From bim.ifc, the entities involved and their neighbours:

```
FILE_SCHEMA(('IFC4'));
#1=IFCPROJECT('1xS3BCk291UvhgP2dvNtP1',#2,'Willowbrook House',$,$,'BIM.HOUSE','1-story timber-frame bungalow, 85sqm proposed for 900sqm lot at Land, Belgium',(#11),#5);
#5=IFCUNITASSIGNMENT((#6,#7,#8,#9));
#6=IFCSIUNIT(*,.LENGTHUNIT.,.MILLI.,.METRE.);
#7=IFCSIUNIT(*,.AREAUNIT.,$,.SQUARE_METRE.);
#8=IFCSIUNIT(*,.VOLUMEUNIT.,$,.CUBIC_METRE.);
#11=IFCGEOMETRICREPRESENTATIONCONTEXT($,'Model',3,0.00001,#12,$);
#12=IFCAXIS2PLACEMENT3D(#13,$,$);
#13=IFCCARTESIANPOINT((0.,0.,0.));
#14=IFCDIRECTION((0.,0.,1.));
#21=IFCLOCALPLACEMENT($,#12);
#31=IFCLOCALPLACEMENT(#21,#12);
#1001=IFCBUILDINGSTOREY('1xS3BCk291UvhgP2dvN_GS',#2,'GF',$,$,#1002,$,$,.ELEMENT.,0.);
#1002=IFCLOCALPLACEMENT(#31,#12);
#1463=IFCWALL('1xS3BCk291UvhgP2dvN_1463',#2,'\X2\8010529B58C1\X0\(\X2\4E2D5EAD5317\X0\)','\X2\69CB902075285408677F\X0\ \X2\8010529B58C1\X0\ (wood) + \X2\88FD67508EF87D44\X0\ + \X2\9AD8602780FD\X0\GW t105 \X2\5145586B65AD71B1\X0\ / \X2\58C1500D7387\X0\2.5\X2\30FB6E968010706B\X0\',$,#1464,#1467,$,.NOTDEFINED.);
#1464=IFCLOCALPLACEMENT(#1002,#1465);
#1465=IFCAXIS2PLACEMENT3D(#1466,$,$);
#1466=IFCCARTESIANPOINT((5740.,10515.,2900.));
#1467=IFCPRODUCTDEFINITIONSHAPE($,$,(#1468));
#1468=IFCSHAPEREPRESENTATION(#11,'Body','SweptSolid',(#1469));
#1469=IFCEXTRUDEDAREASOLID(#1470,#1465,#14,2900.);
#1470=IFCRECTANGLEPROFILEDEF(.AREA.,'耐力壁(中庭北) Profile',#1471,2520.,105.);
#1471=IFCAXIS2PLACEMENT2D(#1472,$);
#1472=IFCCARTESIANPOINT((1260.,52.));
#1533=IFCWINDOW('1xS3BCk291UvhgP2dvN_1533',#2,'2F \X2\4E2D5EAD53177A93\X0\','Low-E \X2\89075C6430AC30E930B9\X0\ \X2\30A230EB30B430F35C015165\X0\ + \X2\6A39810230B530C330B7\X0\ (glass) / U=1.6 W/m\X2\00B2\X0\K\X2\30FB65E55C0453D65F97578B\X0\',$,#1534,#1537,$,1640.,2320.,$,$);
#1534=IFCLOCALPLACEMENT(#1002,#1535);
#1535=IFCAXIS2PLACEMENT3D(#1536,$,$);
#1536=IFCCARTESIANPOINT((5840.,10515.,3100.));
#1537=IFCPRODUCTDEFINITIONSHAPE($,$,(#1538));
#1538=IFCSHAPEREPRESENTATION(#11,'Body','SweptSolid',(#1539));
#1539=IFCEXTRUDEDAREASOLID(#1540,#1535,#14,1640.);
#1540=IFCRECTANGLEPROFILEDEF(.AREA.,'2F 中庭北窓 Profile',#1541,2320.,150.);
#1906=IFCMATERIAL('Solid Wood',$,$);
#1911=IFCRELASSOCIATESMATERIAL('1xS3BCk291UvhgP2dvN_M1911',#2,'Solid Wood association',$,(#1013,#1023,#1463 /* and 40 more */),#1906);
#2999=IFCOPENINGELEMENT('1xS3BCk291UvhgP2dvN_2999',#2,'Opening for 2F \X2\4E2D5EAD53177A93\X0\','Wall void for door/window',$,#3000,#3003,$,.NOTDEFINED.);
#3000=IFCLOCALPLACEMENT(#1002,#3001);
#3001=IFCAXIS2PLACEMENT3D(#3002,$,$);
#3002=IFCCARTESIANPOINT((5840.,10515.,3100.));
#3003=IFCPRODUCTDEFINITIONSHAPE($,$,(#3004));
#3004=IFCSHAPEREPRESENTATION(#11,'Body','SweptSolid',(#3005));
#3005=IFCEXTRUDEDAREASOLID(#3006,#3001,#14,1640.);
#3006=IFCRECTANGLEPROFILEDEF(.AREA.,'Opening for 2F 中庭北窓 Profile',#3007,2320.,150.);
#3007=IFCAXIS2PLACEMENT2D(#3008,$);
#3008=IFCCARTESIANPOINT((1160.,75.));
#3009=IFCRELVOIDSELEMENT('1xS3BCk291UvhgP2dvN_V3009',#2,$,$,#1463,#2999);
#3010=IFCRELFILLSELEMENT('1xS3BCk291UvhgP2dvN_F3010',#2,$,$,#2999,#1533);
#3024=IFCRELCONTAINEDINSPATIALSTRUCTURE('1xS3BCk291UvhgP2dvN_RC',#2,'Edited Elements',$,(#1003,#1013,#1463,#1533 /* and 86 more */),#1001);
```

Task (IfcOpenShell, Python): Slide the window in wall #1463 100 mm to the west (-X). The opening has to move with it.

```python
import ifcopenshell
import ifcopenshell.api.geometry
import ifcopenshell.util.placement

model = ifcopenshell.open("bim.ifc")

window = model.by_id(1533)
opening = window.FillsVoids[0].RelatingOpeningElement
wall = opening.VoidsElements[0].RelatingBuildingElement

wall_matrix = ifcopenshell.util.placement.get_local_placement(wall.ObjectPlacement)
shift = wall_matrix[:3, 0] * -100.0
before = ifcopenshell.util.placement.get_local_placement(window.ObjectPlacement)[:3, 3].copy()

# The window is not placed relative to its opening, so move both.
for product in (opening, window):
    matrix = ifcopenshell.util.placement.get_local_placement(product.ObjectPlacement)
    matrix[:3, 3] += shift
    ifcopenshell.api.geometry.edit_object_placement(model, product=product, matrix=matrix, is_si=False)

after = ifcopenshell.util.placement.get_local_placement(window.ObjectPlacement)[:3, 3]
print("window moved by", (after - before).round(3) + 0.0)

model.write("bim_updated.ifc")
```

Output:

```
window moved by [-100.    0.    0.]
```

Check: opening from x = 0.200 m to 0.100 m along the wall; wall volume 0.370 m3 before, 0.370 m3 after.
